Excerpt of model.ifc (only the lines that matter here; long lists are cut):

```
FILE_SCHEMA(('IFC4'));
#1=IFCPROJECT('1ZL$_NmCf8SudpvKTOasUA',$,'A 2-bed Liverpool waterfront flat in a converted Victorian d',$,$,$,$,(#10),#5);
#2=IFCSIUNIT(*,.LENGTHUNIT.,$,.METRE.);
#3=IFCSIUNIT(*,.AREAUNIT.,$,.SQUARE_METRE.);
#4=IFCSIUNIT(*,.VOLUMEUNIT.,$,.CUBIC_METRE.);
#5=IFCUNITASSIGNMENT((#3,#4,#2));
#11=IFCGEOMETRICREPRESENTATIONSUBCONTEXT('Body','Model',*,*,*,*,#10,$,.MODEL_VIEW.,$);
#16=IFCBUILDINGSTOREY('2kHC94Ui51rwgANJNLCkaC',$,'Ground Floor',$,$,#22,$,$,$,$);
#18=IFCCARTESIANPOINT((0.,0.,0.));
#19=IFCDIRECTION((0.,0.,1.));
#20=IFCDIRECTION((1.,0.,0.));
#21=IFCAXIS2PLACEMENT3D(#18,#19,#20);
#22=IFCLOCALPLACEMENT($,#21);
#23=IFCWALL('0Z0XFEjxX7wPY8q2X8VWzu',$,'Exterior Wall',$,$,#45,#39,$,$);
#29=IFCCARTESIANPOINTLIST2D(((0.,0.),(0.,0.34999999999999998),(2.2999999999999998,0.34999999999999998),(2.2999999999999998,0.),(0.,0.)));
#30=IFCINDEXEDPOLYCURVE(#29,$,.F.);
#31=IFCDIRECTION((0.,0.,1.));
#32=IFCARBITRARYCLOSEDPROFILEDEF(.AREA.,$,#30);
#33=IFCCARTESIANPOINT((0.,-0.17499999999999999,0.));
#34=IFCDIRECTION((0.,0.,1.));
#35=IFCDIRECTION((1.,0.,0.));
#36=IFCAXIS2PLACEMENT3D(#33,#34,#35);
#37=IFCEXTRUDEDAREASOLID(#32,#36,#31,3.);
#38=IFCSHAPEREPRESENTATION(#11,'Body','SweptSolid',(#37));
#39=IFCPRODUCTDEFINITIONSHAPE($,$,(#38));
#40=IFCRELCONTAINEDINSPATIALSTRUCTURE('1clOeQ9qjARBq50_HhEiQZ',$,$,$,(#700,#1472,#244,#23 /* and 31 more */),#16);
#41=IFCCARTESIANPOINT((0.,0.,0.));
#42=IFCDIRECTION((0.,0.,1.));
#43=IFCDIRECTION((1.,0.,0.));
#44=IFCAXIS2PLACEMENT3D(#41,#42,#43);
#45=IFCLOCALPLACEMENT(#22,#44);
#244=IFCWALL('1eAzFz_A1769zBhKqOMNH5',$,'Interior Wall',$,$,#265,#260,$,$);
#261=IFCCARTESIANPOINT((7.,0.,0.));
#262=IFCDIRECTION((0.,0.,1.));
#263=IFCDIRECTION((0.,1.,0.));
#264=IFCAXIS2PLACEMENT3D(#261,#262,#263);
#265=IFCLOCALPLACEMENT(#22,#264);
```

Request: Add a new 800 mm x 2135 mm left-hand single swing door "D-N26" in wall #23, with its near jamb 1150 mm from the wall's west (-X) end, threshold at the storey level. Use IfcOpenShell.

```python
import numpy as np
import ifcopenshell
import ifcopenshell.api.feature
import ifcopenshell.api.geometry
import ifcopenshell.api.root
import ifcopenshell.api.spatial
import ifcopenshell.geom
import ifcopenshell.util.element
import ifcopenshell.util.placement
import ifcopenshell.util.representation
import ifcopenshell.util.shape
import ifcopenshell.util.unit

model = ifcopenshell.open("model.ifc")
unit_scale = ifcopenshell.util.unit.calculate_unit_scale(model)
settings = ifcopenshell.geom.settings()


def volume(element):
    """Net volume in cubic metres, openings subtracted."""
    shape = ifcopenshell.geom.create_shape(settings, element)
    return ifcopenshell.util.shape.get_volume(shape.geometry)


wall = model.by_id(23)
storey = ifcopenshell.util.element.get_container(wall, ifc_class="IfcBuildingStorey")
context = ifcopenshell.util.representation.get_context(model, "Model", "Body", "MODEL_VIEW")
before = volume(wall)

width, height, from_end, sill = 0.8, 2.135, 1.15, 0.0  # metres

# The wall runs along its own X axis, and the end named is its -X end.
wall_shape = ifcopenshell.geom.create_shape(settings, wall)
x, y, z = ifcopenshell.util.shape.get_vertices(wall_shape.geometry).T
start = x.min() + from_end
face, thickness = float(y.min()), float(y.max() - y.min())
wall_matrix = ifcopenshell.util.placement.get_local_placement(wall.ObjectPlacement)
level = ifcopenshell.util.placement.get_local_placement(storey.ObjectPlacement)[2, 3]


def in_wall(x, y):
    """Placement at x, y metres in the wall's axes, at sill height."""
    matrix = wall_matrix.copy()
    matrix[:, 3] = wall_matrix @ np.array([x / unit_scale, y / unit_scale, 0.0, 1.0])
    matrix[2, 3] = level + sill / unit_scale
    return matrix


# Opening: a box that overshoots both wall faces by 50 mm.
opening = ifcopenshell.api.root.create_entity(model, ifc_class="IfcOpeningElement", predefined_type="OPENING")
box = ifcopenshell.api.geometry.add_wall_representation(
    model, context=context, length=width, height=height, thickness=thickness + 0.1
)
ifcopenshell.api.geometry.assign_representation(model, product=opening, representation=box)
ifcopenshell.api.geometry.edit_object_placement(model, product=opening, matrix=in_wall(start, face - 0.05), is_si=False)
ifcopenshell.api.feature.add_feature(model, feature=opening, element=wall)

door = ifcopenshell.api.root.create_entity(model, ifc_class="IfcDoor", name="D-N26", predefined_type="DOOR")
door.OverallWidth, door.OverallHeight = width / unit_scale, height / unit_scale
door.OperationType = "SINGLE_SWING_LEFT"
body = ifcopenshell.api.geometry.add_door_representation(
    model,
    context=context,
    overall_width=door.OverallWidth,
    overall_height=door.OverallHeight,
    operation_type="SINGLE_SWING_LEFT",
    lining_properties={"LiningDepth": thickness / unit_scale, "ThresholdDepth": thickness / unit_scale},
)
ifcopenshell.api.geometry.assign_representation(model, product=door, representation=body)
ifcopenshell.api.spatial.assign_container(model, products=[door], relating_structure=storey)
ifcopenshell.api.feature.add_filling(model, opening=opening, element=door)

# The lining spans the wall, so the door starts at the wall face.
ifcopenshell.api.geometry.edit_object_placement(model, product=door, matrix=in_wall(start, face), is_si=False)

after = volume(wall)

print(f"wall volume {before:.3f} -> {after:.3f} m3")

model.write("model_edited.ifc")
```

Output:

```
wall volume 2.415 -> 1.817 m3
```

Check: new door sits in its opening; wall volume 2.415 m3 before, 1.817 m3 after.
